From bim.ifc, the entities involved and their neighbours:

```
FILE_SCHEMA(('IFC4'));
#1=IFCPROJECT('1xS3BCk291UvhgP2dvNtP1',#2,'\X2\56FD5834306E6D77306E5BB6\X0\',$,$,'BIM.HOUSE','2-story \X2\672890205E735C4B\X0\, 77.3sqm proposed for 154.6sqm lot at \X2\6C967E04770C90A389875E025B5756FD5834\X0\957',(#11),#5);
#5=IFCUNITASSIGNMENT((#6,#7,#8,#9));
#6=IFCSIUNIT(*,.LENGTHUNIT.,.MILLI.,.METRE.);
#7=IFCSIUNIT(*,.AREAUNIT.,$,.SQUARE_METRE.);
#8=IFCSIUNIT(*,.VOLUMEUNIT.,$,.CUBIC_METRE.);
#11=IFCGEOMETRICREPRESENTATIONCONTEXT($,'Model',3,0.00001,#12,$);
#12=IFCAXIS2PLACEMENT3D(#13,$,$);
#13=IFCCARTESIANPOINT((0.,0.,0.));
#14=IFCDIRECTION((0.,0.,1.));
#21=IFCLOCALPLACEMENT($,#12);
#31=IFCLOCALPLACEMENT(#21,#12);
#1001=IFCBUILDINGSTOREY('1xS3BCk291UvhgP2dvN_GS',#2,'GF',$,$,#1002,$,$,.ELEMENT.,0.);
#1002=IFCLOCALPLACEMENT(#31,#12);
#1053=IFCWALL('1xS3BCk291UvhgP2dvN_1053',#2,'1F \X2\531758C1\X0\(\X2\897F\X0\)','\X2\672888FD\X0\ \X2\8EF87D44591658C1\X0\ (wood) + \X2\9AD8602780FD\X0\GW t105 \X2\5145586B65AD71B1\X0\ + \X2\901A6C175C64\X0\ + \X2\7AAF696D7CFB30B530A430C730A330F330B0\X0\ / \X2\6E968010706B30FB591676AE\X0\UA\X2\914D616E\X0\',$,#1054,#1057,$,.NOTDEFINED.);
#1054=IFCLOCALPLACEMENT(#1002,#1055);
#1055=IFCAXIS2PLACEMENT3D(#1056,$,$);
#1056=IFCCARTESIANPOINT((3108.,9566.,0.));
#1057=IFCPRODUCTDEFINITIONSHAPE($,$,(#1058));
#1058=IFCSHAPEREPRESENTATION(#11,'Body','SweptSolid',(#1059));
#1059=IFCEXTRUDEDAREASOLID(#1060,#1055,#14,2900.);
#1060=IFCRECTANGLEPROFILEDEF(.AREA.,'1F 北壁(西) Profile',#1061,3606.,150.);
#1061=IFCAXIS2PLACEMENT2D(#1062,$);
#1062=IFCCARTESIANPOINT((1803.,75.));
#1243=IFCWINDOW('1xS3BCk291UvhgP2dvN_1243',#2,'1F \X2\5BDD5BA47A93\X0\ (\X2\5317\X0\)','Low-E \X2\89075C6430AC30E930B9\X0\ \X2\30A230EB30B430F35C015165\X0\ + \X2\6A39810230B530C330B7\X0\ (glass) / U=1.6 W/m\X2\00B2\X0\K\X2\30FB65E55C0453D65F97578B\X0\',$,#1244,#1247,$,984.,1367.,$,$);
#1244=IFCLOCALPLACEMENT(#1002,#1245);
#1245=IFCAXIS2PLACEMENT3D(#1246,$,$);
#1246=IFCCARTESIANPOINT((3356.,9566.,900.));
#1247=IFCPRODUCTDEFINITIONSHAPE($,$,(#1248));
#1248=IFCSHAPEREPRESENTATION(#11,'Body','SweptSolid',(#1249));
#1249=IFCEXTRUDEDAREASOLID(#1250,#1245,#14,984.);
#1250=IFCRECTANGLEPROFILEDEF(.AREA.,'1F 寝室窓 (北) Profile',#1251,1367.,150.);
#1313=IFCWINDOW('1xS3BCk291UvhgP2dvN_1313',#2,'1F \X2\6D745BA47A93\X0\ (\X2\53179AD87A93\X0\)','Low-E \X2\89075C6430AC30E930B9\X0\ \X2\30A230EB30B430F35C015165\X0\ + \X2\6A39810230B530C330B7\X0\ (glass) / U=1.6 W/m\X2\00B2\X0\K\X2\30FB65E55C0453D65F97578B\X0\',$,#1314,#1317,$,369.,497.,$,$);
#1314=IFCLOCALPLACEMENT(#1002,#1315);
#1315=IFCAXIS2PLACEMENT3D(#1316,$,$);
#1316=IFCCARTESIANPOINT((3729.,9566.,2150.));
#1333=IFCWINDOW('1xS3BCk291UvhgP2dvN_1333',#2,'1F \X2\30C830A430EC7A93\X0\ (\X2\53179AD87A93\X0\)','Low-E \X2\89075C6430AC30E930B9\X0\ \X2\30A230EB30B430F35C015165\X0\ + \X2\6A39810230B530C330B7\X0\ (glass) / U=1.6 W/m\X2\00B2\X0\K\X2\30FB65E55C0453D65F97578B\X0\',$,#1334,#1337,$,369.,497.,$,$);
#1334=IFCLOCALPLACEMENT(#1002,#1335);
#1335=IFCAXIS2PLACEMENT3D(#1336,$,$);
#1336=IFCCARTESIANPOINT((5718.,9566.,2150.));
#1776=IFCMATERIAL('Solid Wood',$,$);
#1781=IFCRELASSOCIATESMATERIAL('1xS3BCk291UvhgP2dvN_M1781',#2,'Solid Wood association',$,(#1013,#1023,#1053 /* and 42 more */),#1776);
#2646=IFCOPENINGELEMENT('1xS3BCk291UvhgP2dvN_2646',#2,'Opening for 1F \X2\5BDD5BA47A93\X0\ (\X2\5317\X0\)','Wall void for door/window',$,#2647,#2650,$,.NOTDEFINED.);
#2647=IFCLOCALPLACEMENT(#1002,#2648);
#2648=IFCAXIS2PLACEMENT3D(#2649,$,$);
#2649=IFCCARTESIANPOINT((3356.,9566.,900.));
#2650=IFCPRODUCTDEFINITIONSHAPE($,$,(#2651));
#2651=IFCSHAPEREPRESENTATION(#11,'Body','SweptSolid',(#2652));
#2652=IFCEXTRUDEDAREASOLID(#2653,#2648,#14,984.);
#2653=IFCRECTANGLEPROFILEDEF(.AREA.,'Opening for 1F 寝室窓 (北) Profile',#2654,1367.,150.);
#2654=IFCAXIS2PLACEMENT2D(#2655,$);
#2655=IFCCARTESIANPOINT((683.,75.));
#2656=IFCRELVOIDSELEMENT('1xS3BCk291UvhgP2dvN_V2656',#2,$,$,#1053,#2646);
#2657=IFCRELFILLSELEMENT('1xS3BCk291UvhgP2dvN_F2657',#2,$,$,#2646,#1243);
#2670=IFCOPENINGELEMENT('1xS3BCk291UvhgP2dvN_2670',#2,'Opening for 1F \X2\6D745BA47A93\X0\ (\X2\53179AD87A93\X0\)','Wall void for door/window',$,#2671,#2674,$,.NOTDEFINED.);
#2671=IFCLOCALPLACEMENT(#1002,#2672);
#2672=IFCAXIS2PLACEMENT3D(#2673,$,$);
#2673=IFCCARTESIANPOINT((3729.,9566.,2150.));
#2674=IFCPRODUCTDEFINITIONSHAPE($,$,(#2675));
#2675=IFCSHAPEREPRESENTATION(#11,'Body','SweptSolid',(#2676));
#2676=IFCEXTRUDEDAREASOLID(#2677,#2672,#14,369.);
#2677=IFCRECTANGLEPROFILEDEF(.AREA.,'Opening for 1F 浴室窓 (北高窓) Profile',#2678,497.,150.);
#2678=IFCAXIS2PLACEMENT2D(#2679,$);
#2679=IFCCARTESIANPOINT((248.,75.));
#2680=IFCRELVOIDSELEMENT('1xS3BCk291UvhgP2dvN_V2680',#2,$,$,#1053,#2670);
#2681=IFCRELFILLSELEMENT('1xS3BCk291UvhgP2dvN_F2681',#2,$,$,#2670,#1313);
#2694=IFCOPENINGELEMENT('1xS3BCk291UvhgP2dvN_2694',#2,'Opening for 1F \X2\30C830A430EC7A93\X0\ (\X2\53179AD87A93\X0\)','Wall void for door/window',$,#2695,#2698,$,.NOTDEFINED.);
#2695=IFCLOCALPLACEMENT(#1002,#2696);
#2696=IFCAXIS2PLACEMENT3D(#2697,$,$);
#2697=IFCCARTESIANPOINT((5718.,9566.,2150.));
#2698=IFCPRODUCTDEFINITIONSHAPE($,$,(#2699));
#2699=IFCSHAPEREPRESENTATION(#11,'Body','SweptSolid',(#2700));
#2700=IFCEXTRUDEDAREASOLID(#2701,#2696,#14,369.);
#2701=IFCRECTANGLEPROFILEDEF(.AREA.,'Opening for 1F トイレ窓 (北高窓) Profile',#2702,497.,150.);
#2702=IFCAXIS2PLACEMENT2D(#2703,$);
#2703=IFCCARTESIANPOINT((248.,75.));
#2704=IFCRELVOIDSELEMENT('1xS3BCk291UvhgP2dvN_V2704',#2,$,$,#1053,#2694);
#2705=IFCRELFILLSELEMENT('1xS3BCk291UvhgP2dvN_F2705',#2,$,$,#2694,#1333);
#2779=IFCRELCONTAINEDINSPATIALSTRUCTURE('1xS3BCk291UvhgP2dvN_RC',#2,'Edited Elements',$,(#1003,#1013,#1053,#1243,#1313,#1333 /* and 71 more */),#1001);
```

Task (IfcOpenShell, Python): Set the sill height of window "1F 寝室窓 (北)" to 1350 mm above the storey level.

```python
import numpy as np
import ifcopenshell
import ifcopenshell.api.geometry
import ifcopenshell.geom
import ifcopenshell.util.element
import ifcopenshell.util.placement
import ifcopenshell.util.shape
import ifcopenshell.util.unit

model = ifcopenshell.open("bim.ifc")
unit_scale = ifcopenshell.util.unit.calculate_unit_scale(model)

window = model.by_guid("1xS3BCk291UvhgP2dvN_1243")
opening = window.FillsVoids[0].RelatingOpeningElement
storey = ifcopenshell.util.element.get_container(window, ifc_class="IfcBuildingStorey")
level = ifcopenshell.util.placement.get_local_placement(storey.ObjectPlacement)[2, 3]

# The opening's origin need not be at the sill, so measure its lowest point.
shape = ifcopenshell.geom.create_shape(ifcopenshell.geom.settings(), opening)
bottom = ifcopenshell.util.shape.get_shape_bottom_elevation(shape, shape.geometry) / unit_scale
dz = level + 1.35 / unit_scale - bottom

shift = np.array([0.0, 0.0, dz])
# The window is not placed relative to its opening, so move both.
for product in (opening, window):
    matrix = ifcopenshell.util.placement.get_local_placement(product.ObjectPlacement)
    matrix[:3, 3] += shift
    ifcopenshell.api.geometry.edit_object_placement(model, product=product, matrix=matrix, is_si=False)

print(f"moved by {dz * unit_scale:+.3f} m")

model.write("bim_edited.ifc")
```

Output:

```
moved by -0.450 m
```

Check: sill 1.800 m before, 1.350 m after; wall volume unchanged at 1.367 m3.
